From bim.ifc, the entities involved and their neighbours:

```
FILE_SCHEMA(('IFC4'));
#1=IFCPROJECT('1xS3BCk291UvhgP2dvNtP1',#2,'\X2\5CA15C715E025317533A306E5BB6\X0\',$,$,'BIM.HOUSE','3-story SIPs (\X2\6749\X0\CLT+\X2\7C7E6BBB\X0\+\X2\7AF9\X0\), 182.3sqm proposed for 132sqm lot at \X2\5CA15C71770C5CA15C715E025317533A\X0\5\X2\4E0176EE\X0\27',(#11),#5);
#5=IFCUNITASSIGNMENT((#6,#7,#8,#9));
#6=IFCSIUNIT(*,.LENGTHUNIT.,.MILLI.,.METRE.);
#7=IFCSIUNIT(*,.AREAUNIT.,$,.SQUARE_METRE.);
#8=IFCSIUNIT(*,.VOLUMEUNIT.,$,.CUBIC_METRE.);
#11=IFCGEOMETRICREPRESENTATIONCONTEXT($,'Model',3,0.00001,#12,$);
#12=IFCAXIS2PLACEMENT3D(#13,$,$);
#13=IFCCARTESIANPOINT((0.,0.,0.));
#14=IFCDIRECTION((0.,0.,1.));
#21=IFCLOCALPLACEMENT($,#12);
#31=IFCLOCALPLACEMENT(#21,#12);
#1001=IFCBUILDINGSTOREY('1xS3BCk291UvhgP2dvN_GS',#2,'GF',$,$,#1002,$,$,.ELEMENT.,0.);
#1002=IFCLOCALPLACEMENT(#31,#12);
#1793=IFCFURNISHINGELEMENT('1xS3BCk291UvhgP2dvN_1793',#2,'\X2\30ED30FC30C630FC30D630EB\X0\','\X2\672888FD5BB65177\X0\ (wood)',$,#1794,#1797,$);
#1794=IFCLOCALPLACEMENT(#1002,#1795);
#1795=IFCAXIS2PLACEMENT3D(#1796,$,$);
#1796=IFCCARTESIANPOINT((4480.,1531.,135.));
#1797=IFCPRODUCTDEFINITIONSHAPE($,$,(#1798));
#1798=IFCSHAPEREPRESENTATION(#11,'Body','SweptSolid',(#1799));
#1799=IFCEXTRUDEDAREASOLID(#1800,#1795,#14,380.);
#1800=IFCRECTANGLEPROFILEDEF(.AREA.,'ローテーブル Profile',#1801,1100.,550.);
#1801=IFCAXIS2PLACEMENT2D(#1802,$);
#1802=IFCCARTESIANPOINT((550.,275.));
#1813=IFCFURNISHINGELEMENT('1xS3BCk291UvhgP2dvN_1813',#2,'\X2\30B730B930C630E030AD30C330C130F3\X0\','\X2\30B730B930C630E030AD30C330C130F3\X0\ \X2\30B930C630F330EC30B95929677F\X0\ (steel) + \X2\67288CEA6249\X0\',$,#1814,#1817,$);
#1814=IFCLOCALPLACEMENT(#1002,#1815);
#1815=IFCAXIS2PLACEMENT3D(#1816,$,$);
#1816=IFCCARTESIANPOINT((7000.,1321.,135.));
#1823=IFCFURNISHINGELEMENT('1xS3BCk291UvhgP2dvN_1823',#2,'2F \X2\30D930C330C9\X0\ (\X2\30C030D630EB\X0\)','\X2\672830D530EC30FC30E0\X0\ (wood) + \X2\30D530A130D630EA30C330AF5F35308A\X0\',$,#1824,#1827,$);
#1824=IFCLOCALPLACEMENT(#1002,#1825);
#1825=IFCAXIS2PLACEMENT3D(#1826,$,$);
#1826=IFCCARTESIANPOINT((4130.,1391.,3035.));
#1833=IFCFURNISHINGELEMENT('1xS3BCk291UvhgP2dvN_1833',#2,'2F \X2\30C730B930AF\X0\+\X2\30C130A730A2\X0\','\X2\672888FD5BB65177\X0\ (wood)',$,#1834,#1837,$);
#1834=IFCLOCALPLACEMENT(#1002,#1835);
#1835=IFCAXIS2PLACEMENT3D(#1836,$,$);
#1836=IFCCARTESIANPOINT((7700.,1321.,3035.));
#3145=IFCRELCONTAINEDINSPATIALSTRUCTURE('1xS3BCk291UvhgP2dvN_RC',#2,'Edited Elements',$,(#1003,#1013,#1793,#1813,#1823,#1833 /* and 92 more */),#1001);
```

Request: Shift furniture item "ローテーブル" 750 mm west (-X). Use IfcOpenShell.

```python
import ifcopenshell
import ifcopenshell.api.geometry
import ifcopenshell.util.placement
import ifcopenshell.util.unit

model = ifcopenshell.open("bim.ifc")
unit_scale = ifcopenshell.util.unit.calculate_unit_scale(model)

item = model.by_guid("1xS3BCk291UvhgP2dvN_1793")
matrix = ifcopenshell.util.placement.get_local_placement(item.ObjectPlacement)
matrix[0, 3] -= 0.75 / unit_scale
ifcopenshell.api.geometry.edit_object_placement(model, product=item, matrix=matrix, is_si=False)

print(ifcopenshell.util.placement.get_local_placement(item.ObjectPlacement).round(3) + 0.0)

model.write("bim-out.ifc")
```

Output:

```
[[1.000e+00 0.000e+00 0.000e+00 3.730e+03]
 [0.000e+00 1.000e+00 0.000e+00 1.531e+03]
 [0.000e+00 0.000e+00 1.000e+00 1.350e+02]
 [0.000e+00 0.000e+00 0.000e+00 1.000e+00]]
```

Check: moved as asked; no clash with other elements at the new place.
